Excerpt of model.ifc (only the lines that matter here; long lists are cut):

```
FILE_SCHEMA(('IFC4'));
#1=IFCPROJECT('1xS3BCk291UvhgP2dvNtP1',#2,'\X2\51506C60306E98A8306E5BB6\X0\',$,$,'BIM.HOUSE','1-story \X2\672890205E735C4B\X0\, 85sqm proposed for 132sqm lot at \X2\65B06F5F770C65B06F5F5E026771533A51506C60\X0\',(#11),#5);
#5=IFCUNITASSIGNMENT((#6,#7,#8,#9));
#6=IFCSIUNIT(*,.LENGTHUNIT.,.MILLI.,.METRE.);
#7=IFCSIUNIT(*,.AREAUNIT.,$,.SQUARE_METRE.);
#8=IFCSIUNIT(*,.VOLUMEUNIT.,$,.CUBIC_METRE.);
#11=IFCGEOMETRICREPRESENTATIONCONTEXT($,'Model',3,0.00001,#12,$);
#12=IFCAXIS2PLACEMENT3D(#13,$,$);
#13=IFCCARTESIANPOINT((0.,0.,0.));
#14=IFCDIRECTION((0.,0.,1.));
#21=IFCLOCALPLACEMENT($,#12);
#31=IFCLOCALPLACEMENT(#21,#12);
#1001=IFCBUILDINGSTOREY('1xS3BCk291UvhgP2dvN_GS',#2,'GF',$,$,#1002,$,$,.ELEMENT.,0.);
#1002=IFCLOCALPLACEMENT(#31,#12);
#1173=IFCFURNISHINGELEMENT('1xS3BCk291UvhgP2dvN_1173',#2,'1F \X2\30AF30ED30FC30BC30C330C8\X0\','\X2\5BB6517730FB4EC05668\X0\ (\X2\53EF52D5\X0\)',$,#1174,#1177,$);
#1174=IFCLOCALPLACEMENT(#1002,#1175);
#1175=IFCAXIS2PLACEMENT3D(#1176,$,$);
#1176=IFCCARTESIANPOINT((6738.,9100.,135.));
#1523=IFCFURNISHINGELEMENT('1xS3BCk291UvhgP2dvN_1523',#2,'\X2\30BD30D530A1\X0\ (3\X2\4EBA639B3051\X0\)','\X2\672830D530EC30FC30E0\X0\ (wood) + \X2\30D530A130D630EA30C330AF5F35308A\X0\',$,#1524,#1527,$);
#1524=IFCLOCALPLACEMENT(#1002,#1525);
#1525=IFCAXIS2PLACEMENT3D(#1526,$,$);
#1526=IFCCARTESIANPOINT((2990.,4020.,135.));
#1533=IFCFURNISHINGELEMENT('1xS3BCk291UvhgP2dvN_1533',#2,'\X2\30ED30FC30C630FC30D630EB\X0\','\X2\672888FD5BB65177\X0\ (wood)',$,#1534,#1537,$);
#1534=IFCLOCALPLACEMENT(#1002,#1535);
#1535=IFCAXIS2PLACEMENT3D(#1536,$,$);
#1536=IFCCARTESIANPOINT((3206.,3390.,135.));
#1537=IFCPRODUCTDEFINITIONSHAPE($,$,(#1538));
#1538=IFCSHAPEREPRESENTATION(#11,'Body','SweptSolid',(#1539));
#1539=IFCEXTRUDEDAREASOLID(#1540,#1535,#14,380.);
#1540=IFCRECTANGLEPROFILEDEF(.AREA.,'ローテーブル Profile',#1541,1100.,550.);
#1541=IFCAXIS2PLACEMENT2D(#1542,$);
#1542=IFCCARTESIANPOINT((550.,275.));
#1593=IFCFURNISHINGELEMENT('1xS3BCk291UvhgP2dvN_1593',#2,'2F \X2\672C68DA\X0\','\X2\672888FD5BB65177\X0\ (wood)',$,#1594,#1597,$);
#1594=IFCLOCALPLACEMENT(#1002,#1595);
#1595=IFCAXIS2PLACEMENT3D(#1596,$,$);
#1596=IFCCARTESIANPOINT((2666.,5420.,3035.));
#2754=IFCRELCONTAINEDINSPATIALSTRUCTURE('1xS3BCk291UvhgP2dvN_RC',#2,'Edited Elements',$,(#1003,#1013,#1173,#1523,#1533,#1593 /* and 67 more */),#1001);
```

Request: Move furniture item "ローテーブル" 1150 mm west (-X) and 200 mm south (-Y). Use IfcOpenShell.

```python
import ifcopenshell
import ifcopenshell.api.geometry
import ifcopenshell.util.placement
import ifcopenshell.util.unit

model = ifcopenshell.open("model.ifc")
unit_scale = ifcopenshell.util.unit.calculate_unit_scale(model)

item = model.by_id(1533)
matrix = ifcopenshell.util.placement.get_local_placement(item.ObjectPlacement)
matrix[0, 3] -= 1.15 / unit_scale
matrix[1, 3] -= 0.2 / unit_scale
ifcopenshell.api.geometry.edit_object_placement(model, product=item, matrix=matrix, is_si=False)

print(ifcopenshell.util.placement.get_local_placement(item.ObjectPlacement).round(3) + 0.0)

model.write("model_v2.ifc")
```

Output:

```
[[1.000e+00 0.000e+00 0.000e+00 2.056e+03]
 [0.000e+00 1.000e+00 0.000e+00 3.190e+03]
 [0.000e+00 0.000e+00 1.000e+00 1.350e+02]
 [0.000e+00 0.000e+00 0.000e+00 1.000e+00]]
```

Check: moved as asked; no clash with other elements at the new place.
